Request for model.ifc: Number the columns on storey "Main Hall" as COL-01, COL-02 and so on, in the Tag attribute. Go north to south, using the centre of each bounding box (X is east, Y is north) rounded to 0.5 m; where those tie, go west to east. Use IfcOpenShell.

First a look at what the model holds.

```python
import ifcopenshell
import ifcopenshell.util.element
import ifcopenshell.util.placement

model = ifcopenshell.open("model.ifc")
print(model.schema)
storey = next(s for s in model.by_type("IfcBuildingStorey") if s.Name == "Main Hall")
columns = [e for e in ifcopenshell.util.element.get_decomposition(storey) if e.is_a("IfcColumn")]
for e in sorted(columns, key=lambda e: e.id()):
    origin = ifcopenshell.util.placement.get_local_placement(e.ObjectPlacement)[:3, 3]
    print(e.id(), e.Tag, e.Name, origin.round(2) + 0.0, sep=" | ")
```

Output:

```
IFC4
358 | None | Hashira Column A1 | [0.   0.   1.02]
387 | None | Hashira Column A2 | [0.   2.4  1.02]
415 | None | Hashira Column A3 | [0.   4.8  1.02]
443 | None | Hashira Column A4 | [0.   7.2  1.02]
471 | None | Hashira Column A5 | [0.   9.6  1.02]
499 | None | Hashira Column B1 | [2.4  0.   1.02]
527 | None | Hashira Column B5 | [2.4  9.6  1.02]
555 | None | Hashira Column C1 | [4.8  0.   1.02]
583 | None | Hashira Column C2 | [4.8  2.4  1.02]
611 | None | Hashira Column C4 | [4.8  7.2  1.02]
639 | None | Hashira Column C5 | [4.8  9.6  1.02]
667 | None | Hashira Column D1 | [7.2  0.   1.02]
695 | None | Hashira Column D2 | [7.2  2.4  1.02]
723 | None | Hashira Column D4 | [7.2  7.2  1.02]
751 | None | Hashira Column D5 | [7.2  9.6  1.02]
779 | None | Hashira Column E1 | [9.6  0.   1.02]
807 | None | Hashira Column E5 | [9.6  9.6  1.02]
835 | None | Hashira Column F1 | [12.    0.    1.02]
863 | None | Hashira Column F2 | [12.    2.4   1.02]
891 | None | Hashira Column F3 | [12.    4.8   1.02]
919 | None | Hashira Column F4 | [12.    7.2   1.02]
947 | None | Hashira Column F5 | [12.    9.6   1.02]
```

```python
import ifcopenshell
import ifcopenshell.geom
import ifcopenshell.util.element
import ifcopenshell.util.shape

model = ifcopenshell.open("model.ifc")
settings = ifcopenshell.geom.settings()
settings.set("use-world-coords", True)


def centre(element):
    shape = ifcopenshell.geom.create_shape(settings, element)
    return ifcopenshell.util.shape.get_bbox_centroid(shape.geometry)


storey = next(s for s in model.by_type("IfcBuildingStorey") if s.Name == "Main Hall")
columns = [e for e in ifcopenshell.util.element.get_decomposition(storey) if e.is_a("IfcColumn")]

# Insertion points can sit at a corner or the storey origin, so sort by the geometry (in metres).
centres = {e: centre(e) for e in columns}
columns.sort(key=lambda e: (-round(centres[e][1] / 0.5), centres[e][0]))

for i, e in enumerate(columns, start=1):
    number = f"COL-{i:02d}"
    e.Tag = number
    print(e.id(), number)

model.write("model_v2.ifc")
```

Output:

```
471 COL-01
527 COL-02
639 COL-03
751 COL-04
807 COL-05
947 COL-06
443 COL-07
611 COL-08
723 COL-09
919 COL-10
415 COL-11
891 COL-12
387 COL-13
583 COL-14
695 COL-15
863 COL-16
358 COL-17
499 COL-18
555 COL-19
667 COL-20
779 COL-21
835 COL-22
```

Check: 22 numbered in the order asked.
